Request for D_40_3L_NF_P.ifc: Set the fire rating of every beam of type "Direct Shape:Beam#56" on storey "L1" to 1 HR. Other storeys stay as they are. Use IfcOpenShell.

First a look at what the model holds.

```python
import ifcopenshell
import ifcopenshell.util.element

model = ifcopenshell.open("D_40_3L_NF_P.ifc")
print(model.schema)
storey = next(s for s in model.by_type("IfcBuildingStorey") if s.Name == "L1")
beams = [e for e in ifcopenshell.util.element.get_decomposition(storey) if e.is_a("IfcBeam")]
seen = {}
for e in beams:
    element_type = ifcopenshell.util.element.get_type(e)
    key = (element_type.Name if element_type != e and element_type else None, ifcopenshell.util.element.get_pset(e, "Pset_BeamCommon", "FireRating"))
    seen[key] = seen.get(key, 0) + 1
for (name, value), count in sorted(seen.items(), key=str):
    print(count, "x", name, "|", value)
```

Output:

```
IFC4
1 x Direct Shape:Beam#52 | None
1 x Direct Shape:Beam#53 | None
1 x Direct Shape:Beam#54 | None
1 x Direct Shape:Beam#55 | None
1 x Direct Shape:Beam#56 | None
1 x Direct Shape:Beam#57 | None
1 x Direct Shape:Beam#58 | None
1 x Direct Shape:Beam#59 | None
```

```python
import ifcopenshell
import ifcopenshell.api.pset
import ifcopenshell.util.element

model = ifcopenshell.open("D_40_3L_NF_P.ifc")

storey = next(s for s in model.by_type("IfcBuildingStorey") if s.Name == "L1")
beams = [e for e in ifcopenshell.util.element.get_decomposition(storey) if e.is_a("IfcBeam")]

count = 0
for e in beams:
    element_type = ifcopenshell.util.element.get_type(e)
    if element_type in (None, e) or element_type.Name != "Direct Shape:Beam#56":
        continue
    # add_pset returns the element's existing set when there is one.
    pset = ifcopenshell.api.pset.add_pset(model, product=e, name="Pset_BeamCommon")
    ifcopenshell.api.pset.edit_pset(model, pset=pset, properties={"FireRating": "1 HR"})
    count += 1

print(count, "beams updated")

model.write("D_40_3L_NF_P_updated.ifc")
```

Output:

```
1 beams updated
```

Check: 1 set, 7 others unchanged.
